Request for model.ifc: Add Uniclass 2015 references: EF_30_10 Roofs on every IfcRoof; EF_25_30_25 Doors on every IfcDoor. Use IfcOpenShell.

First a look at what the model holds.

```python
import ifcopenshell

model = ifcopenshell.open("model.ifc")
print(model.schema)
print("classifications:", [c.Name for c in model.by_type("IfcClassification")])
for ifc_class in ("IfcDoor", "IfcRoof", "IfcStair", "IfcWall", "IfcWindow"):
    print(ifc_class, len(model.by_type(ifc_class)))
```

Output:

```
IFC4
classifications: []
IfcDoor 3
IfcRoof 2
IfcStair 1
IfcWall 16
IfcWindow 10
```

```python
import ifcopenshell
import ifcopenshell.api.classification

model = ifcopenshell.open("model.ifc")

system = ifcopenshell.api.classification.add_classification(model, classification="Uniclass 2015")

codes = {
    "IfcRoof": ("EF_30_10", "Roofs"),
    "IfcDoor": ("EF_25_30_25", "Doors"),
}
for ifc_class, (code, name) in codes.items():
    products = model.by_type(ifc_class)
    ifcopenshell.api.classification.add_reference(
        model, products=products, classification=system, identification=code, name=name
    )
    print(code, len(products))

model.write("model_updated.ifc")
```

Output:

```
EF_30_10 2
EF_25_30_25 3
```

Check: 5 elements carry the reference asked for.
